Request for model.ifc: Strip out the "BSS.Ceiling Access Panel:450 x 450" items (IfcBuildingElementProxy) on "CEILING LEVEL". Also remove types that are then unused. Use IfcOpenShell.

First a look at what the model holds.

```python
import ifcopenshell
import ifcopenshell.util.element

model = ifcopenshell.open("model.ifc")
print(model.schema)
storey = next(s for s in model.by_type("IfcBuildingStorey") if s.Name == "CEILING LEVEL")
proxies = [e for e in ifcopenshell.util.element.get_decomposition(storey) if e.is_a("IfcBuildingElementProxy")]
seen = {}
for e in proxies:
    element_type = ifcopenshell.util.element.get_type(e)
    name = element_type.Name if element_type not in (None, e) else None
    seen[name] = seen.get(name, 0) + 1
for name, count in sorted(seen.items(), key=str):
    print(count, "x", name)
```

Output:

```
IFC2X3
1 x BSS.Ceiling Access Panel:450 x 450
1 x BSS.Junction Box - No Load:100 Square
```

```python
import ifcopenshell
import ifcopenshell.api.root
import ifcopenshell.util.element

model = ifcopenshell.open("model.ifc")

storey = next(s for s in model.by_type("IfcBuildingStorey") if s.Name == "CEILING LEVEL")
proxies = [e for e in ifcopenshell.util.element.get_decomposition(storey) if e.is_a("IfcBuildingElementProxy")]
targets = [e for e in proxies if (t := ifcopenshell.util.element.get_type(e)) not in (None, e) and t.Name == "BSS.Ceiling Access Panel:450 x 450"]
types = {ifcopenshell.util.element.get_type(e) for e in targets} - {None, *targets}

for e in targets:
    ifcopenshell.api.root.remove_product(model, product=e)
print(len(targets), "removed")

unused = [t for t in types if not ifcopenshell.util.element.get_types(t)]
for t in unused:
    ifcopenshell.api.root.remove_product(model, product=t)
print(len(unused), "unused types removed")

model.write("model_v2.ifc")
```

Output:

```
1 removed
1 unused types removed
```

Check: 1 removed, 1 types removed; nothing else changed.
